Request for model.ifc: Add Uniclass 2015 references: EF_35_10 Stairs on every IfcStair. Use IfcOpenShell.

First a look at what the model holds.

```python
import ifcopenshell

model = ifcopenshell.open("model.ifc")
print(model.schema)
print("classifications:", [c.Name for c in model.by_type("IfcClassification")])
for ifc_class in ("IfcDoor", "IfcRoof", "IfcStair", "IfcWall", "IfcWindow"):
    print(ifc_class, len(model.by_type(ifc_class)))
```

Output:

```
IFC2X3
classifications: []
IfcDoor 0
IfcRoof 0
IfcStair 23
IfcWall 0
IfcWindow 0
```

```python
import ifcopenshell
import ifcopenshell.api.classification

model = ifcopenshell.open("model.ifc")

# IFC2X3 requires Source and Edition and has no link from the project to the system.
system = model.create_entity("IfcClassification", Source="NBS", Edition="2015", Name="Uniclass 2015")

codes = {
    "IfcStair": ("EF_35_10", "Stairs"),
}
for ifc_class, (code, name) in codes.items():
    products = model.by_type(ifc_class)
    ifcopenshell.api.classification.add_reference(
        model, products=products, classification=system, identification=code, name=name
    )
    print(code, len(products))

model.write("model_edited.ifc")
```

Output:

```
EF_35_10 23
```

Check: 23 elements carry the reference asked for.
